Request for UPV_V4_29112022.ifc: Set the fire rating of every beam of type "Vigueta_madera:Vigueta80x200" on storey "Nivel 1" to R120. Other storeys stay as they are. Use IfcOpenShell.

First a look at what the model holds.

```python
import ifcopenshell
import ifcopenshell.util.element

model = ifcopenshell.open("UPV_V4_29112022.ifc")
print(model.schema)
storey = next(s for s in model.by_type("IfcBuildingStorey") if s.Name == "Nivel 1")
beams = [e for e in ifcopenshell.util.element.get_decomposition(storey) if e.is_a("IfcBeam")]
seen = {}
for e in beams:
    element_type = ifcopenshell.util.element.get_type(e)
    key = (element_type.Name if element_type != e and element_type else None, ifcopenshell.util.element.get_pset(e, "Pset_BeamCommon", "FireRating"))
    seen[key] = seen.get(key, 0) + 1
for (name, value), count in sorted(seen.items(), key=str):
    print(count, "x", name, "|", value)
```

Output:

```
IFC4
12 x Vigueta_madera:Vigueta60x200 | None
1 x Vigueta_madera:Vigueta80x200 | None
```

```python
import ifcopenshell
import ifcopenshell.api.pset
import ifcopenshell.util.element

model = ifcopenshell.open("UPV_V4_29112022.ifc")

storey = next(s for s in model.by_type("IfcBuildingStorey") if s.Name == "Nivel 1")
beams = [e for e in ifcopenshell.util.element.get_decomposition(storey) if e.is_a("IfcBeam")]

count = 0
for e in beams:
    element_type = ifcopenshell.util.element.get_type(e)
    if element_type in (None, e) or element_type.Name != "Vigueta_madera:Vigueta80x200":
        continue
    # add_pset returns the element's existing set when there is one.
    pset = ifcopenshell.api.pset.add_pset(model, product=e, name="Pset_BeamCommon")
    ifcopenshell.api.pset.edit_pset(model, pset=pset, properties={"FireRating": "R120"})
    count += 1

print(count, "beams updated")

model.write("UPV_V4_29112022_rev.ifc")
```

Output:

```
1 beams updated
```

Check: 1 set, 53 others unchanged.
